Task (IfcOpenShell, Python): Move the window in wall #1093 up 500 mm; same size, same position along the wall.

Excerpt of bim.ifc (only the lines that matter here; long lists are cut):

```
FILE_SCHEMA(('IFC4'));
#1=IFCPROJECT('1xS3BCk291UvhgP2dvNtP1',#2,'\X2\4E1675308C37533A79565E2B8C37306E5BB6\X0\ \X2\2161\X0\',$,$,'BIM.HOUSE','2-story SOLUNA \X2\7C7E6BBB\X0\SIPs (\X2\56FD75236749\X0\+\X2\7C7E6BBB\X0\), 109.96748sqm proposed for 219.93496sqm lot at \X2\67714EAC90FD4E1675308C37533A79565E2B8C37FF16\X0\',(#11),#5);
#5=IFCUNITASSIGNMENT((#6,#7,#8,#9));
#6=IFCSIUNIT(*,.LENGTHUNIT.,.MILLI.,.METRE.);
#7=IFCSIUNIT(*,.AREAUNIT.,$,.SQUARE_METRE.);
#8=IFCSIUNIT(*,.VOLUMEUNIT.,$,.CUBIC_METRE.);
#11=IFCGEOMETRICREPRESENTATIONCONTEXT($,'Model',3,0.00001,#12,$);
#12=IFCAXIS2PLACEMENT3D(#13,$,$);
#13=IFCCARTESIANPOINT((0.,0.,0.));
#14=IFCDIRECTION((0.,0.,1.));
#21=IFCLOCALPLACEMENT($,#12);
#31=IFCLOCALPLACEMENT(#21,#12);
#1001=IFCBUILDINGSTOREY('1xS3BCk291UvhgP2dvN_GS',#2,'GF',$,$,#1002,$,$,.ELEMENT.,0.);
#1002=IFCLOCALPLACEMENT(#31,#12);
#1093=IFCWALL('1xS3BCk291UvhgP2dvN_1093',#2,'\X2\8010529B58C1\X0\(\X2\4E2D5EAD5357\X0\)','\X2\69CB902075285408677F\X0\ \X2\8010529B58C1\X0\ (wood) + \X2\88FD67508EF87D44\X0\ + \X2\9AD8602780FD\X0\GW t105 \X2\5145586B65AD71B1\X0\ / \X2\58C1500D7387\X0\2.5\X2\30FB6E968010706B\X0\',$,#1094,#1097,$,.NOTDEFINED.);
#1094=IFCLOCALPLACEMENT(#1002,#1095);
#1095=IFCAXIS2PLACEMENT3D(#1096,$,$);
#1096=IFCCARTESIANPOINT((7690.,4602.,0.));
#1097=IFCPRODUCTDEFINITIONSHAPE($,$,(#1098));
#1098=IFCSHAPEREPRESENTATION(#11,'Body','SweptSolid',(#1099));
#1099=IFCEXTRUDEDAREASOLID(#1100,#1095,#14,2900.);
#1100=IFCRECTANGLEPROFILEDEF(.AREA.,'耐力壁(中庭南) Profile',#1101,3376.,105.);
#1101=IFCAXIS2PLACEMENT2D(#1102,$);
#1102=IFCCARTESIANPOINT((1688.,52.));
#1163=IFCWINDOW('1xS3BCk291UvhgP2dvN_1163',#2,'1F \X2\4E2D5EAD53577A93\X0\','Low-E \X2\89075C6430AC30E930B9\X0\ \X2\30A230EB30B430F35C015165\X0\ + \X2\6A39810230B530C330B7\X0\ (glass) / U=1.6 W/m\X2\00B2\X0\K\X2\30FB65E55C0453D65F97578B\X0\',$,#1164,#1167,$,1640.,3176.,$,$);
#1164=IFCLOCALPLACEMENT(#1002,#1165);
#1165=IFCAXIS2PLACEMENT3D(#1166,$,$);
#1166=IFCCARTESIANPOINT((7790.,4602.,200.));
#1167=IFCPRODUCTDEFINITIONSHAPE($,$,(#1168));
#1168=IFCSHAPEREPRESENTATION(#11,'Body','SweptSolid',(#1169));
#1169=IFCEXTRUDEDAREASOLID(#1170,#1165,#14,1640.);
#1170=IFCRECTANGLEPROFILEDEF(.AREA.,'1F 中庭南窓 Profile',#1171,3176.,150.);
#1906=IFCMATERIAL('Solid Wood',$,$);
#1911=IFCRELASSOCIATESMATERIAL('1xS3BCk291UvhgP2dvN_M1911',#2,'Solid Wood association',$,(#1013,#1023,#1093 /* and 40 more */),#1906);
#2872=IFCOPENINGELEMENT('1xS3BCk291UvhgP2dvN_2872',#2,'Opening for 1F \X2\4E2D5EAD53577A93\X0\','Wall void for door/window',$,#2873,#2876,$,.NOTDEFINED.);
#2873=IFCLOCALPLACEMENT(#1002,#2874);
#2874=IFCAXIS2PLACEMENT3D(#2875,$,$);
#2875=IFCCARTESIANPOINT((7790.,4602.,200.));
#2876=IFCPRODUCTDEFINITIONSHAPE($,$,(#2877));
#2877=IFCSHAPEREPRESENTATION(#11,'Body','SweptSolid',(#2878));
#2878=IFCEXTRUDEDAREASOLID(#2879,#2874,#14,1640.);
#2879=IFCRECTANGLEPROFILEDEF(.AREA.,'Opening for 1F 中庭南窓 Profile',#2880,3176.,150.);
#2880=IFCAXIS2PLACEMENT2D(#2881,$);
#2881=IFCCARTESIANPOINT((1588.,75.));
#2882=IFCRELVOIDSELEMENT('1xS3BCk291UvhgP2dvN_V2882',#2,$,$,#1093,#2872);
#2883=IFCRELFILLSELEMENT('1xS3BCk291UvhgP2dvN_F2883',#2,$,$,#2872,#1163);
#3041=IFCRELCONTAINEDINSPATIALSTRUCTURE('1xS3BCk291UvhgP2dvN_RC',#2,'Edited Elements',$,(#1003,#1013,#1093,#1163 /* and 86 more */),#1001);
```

```python
import numpy as np
import ifcopenshell
import ifcopenshell.api.geometry
import ifcopenshell.util.placement
import ifcopenshell.util.unit

model = ifcopenshell.open("bim.ifc")
unit_scale = ifcopenshell.util.unit.calculate_unit_scale(model)

window = model.by_id(1163)
opening = window.FillsVoids[0].RelatingOpeningElement
dz = 0.5 / unit_scale

shift = np.array([0.0, 0.0, dz])
# The window is not placed relative to its opening, so move both.
for product in (opening, window):
    matrix = ifcopenshell.util.placement.get_local_placement(product.ObjectPlacement)
    matrix[:3, 3] += shift
    ifcopenshell.api.geometry.edit_object_placement(model, product=product, matrix=matrix, is_si=False)

print(f"moved by {dz * unit_scale:+.3f} m")

model.write("bim-out.ifc")
```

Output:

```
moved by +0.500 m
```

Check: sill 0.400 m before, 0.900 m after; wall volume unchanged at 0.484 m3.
